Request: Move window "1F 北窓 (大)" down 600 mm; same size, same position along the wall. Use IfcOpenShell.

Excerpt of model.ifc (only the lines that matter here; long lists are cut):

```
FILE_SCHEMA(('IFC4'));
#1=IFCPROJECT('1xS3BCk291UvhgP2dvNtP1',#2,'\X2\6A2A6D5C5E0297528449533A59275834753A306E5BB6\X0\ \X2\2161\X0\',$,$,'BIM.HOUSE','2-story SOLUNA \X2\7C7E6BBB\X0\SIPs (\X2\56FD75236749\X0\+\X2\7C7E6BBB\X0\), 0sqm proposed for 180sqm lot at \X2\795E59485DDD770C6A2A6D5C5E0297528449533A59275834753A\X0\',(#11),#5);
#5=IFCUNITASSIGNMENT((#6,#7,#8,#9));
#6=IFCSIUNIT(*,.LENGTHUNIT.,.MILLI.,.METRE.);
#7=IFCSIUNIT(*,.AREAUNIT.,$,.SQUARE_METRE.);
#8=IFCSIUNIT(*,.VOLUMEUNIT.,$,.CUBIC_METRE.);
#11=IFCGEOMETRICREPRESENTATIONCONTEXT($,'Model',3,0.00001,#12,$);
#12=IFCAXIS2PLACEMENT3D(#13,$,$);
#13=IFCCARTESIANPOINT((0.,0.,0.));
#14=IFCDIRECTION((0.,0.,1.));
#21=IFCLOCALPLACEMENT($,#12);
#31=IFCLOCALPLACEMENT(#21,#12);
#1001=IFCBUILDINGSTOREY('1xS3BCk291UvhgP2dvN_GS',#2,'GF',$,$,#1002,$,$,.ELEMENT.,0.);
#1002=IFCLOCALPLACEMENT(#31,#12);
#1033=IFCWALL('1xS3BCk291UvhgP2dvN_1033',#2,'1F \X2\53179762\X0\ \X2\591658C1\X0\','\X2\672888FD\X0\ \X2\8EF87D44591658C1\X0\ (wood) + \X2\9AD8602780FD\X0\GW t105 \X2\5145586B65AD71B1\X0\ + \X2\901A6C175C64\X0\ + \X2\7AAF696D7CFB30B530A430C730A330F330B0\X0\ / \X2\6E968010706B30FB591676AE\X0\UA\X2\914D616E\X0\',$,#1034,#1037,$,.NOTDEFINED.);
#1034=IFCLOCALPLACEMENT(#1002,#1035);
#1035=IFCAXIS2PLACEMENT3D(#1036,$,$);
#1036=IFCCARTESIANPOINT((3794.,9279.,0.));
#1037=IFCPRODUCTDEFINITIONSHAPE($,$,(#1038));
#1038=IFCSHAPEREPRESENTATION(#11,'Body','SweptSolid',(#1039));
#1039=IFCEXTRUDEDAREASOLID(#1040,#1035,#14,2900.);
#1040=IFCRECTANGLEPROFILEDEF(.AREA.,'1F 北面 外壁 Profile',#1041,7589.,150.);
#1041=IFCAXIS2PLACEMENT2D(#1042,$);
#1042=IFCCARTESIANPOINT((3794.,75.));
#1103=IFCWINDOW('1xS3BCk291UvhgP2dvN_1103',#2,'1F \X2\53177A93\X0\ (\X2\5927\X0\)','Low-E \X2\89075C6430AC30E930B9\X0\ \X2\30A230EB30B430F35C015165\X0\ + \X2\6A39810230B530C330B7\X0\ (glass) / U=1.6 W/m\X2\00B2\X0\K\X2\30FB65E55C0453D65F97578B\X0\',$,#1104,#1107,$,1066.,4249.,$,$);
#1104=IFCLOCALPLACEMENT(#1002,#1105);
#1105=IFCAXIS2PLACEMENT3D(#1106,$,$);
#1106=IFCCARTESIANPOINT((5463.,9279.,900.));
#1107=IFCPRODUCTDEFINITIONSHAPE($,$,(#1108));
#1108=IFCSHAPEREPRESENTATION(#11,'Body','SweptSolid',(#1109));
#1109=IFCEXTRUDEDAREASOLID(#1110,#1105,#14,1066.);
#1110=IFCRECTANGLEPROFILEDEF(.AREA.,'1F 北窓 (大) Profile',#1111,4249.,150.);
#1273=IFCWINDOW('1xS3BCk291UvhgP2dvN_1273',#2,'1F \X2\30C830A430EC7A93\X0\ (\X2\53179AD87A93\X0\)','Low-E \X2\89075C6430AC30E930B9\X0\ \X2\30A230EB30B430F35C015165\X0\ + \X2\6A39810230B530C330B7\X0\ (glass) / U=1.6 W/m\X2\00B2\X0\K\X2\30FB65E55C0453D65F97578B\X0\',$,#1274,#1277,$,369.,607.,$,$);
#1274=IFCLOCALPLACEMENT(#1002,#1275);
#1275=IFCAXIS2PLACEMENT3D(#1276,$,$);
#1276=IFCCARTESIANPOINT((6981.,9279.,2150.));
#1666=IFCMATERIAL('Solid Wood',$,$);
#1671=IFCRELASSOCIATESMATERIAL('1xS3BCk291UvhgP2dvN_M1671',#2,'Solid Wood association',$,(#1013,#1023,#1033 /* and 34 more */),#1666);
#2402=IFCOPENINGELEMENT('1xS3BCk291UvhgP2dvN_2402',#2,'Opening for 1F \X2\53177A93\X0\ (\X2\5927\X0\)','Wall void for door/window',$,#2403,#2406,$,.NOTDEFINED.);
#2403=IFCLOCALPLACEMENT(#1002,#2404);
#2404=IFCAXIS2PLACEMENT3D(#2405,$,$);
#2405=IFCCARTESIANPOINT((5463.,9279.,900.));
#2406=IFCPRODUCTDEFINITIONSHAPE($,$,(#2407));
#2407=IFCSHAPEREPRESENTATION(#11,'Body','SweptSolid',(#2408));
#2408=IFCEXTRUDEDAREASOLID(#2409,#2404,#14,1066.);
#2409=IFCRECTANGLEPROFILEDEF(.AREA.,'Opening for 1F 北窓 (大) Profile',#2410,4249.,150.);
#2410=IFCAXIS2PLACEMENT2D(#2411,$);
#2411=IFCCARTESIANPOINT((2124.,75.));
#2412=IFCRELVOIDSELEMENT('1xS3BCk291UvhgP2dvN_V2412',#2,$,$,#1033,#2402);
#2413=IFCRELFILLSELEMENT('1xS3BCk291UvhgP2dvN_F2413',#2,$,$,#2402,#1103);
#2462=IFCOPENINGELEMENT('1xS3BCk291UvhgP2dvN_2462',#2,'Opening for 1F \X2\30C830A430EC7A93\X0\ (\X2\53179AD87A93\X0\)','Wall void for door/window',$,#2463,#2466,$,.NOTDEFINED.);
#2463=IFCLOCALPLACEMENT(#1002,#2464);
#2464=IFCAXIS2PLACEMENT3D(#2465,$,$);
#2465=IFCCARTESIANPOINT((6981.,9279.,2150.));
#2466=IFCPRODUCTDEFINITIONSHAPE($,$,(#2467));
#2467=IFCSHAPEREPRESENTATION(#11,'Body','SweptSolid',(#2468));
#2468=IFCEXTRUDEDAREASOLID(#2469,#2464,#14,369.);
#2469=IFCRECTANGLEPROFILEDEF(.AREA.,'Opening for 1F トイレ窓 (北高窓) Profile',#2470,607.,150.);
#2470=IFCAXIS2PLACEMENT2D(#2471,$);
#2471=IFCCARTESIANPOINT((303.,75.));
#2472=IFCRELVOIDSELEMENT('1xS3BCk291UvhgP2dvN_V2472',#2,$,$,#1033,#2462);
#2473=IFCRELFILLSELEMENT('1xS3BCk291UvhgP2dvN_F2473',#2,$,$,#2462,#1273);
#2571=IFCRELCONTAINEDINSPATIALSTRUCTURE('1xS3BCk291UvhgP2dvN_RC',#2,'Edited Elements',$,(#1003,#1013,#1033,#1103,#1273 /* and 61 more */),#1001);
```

```python
import numpy as np
import ifcopenshell
import ifcopenshell.api.geometry
import ifcopenshell.util.placement
import ifcopenshell.util.unit

model = ifcopenshell.open("model.ifc")
unit_scale = ifcopenshell.util.unit.calculate_unit_scale(model)

window = model.by_guid("1xS3BCk291UvhgP2dvN_1103")
opening = window.FillsVoids[0].RelatingOpeningElement
dz = -600.0

shift = np.array([0.0, 0.0, dz])
# The window is not placed relative to its opening, so move both.
for product in (opening, window):
    matrix = ifcopenshell.util.placement.get_local_placement(product.ObjectPlacement)
    matrix[:3, 3] += shift
    ifcopenshell.api.geometry.edit_object_placement(model, product=product, matrix=matrix, is_si=False)

print(f"moved by {dz * unit_scale:+.3f} m")

model.write("model_rev.ifc")
```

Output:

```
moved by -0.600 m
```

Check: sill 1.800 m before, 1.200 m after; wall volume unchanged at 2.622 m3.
